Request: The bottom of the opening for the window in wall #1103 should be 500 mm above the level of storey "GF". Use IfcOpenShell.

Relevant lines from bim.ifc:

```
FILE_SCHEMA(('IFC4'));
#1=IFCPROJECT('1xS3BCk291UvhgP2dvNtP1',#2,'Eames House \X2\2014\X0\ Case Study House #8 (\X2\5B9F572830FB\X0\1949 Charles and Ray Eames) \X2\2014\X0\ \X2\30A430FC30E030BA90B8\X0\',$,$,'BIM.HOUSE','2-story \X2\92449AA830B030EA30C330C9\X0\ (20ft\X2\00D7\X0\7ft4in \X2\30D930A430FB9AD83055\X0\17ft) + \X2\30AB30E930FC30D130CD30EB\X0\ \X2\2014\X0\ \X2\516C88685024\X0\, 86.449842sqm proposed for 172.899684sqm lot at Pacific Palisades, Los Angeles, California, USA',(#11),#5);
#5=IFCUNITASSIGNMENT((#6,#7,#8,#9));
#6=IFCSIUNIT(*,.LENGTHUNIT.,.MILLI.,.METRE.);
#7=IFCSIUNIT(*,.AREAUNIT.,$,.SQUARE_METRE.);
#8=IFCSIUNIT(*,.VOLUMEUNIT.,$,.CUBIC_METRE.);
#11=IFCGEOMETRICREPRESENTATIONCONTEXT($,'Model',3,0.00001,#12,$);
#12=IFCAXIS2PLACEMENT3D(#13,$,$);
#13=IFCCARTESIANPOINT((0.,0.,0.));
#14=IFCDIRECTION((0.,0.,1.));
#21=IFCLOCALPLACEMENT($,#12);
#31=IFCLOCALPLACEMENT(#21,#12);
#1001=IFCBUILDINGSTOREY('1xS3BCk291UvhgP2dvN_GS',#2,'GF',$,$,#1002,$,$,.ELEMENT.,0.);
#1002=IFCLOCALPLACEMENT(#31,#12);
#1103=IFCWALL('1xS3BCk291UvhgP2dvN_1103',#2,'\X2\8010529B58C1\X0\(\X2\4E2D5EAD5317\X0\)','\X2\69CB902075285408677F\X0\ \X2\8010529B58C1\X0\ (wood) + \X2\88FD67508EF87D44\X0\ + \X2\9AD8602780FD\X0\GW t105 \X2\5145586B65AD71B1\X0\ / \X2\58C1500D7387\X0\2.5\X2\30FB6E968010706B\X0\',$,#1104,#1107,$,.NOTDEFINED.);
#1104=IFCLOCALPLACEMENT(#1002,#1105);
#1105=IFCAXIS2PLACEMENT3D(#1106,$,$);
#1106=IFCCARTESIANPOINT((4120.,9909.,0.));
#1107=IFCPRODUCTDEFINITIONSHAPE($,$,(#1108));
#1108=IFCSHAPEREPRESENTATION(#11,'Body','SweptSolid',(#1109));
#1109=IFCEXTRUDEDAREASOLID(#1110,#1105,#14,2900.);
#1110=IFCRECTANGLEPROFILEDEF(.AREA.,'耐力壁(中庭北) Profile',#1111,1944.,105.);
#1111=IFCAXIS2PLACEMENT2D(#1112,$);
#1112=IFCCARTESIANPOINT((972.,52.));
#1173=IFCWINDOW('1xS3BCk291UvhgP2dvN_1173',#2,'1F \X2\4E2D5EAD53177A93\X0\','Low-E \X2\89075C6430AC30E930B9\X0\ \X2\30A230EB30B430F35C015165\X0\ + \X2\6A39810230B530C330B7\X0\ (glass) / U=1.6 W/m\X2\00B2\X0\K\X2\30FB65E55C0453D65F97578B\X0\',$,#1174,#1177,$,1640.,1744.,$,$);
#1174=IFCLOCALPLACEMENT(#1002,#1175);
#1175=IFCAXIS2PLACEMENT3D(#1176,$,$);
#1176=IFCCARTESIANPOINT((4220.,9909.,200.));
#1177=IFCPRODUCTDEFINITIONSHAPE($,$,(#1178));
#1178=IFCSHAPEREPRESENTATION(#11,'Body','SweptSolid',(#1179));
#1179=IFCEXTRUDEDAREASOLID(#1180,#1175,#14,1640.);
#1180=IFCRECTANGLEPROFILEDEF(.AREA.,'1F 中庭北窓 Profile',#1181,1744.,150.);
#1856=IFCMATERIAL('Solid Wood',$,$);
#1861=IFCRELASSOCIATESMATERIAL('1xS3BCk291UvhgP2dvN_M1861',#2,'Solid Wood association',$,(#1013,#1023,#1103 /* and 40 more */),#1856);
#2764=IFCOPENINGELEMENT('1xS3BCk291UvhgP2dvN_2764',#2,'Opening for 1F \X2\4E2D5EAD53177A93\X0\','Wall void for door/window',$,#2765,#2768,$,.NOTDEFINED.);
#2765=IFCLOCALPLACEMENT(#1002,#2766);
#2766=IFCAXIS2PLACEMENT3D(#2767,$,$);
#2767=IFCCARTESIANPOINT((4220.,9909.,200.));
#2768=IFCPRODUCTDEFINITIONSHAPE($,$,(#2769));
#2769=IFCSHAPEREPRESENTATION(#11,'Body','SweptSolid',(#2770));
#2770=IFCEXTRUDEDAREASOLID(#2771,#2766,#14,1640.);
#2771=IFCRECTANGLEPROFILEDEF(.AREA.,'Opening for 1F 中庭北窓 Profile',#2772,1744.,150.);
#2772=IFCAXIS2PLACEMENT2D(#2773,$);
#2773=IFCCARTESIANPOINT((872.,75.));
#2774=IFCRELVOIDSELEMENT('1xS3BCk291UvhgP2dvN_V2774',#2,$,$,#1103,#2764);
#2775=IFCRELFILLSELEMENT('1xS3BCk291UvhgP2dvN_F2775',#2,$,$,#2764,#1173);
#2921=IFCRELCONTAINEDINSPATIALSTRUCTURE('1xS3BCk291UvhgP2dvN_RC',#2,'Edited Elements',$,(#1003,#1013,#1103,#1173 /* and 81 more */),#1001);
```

```python
import numpy as np
import ifcopenshell
import ifcopenshell.api.geometry
import ifcopenshell.geom
import ifcopenshell.util.element
import ifcopenshell.util.placement
import ifcopenshell.util.shape
import ifcopenshell.util.unit

model = ifcopenshell.open("bim.ifc")
unit_scale = ifcopenshell.util.unit.calculate_unit_scale(model)

window = model.by_guid("1xS3BCk291UvhgP2dvN_1173")
opening = window.FillsVoids[0].RelatingOpeningElement
storey = ifcopenshell.util.element.get_container(window, ifc_class="IfcBuildingStorey")
level = ifcopenshell.util.placement.get_local_placement(storey.ObjectPlacement)[2, 3]

# The opening's origin need not be at the sill, so measure its lowest point.
shape = ifcopenshell.geom.create_shape(ifcopenshell.geom.settings(), opening)
bottom = ifcopenshell.util.shape.get_shape_bottom_elevation(shape, shape.geometry) / unit_scale
dz = level + 500.0 - bottom

shift = np.array([0.0, 0.0, dz])
# The window is not placed relative to its opening, so move both.
for product in (opening, window):
    matrix = ifcopenshell.util.placement.get_local_placement(product.ObjectPlacement)
    matrix[:3, 3] += shift
    ifcopenshell.api.geometry.edit_object_placement(model, product=product, matrix=matrix, is_si=False)

print(f"moved by {dz * unit_scale:+.3f} m")

model.write("bim-out.ifc")
```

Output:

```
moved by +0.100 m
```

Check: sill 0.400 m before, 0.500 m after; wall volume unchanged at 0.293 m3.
